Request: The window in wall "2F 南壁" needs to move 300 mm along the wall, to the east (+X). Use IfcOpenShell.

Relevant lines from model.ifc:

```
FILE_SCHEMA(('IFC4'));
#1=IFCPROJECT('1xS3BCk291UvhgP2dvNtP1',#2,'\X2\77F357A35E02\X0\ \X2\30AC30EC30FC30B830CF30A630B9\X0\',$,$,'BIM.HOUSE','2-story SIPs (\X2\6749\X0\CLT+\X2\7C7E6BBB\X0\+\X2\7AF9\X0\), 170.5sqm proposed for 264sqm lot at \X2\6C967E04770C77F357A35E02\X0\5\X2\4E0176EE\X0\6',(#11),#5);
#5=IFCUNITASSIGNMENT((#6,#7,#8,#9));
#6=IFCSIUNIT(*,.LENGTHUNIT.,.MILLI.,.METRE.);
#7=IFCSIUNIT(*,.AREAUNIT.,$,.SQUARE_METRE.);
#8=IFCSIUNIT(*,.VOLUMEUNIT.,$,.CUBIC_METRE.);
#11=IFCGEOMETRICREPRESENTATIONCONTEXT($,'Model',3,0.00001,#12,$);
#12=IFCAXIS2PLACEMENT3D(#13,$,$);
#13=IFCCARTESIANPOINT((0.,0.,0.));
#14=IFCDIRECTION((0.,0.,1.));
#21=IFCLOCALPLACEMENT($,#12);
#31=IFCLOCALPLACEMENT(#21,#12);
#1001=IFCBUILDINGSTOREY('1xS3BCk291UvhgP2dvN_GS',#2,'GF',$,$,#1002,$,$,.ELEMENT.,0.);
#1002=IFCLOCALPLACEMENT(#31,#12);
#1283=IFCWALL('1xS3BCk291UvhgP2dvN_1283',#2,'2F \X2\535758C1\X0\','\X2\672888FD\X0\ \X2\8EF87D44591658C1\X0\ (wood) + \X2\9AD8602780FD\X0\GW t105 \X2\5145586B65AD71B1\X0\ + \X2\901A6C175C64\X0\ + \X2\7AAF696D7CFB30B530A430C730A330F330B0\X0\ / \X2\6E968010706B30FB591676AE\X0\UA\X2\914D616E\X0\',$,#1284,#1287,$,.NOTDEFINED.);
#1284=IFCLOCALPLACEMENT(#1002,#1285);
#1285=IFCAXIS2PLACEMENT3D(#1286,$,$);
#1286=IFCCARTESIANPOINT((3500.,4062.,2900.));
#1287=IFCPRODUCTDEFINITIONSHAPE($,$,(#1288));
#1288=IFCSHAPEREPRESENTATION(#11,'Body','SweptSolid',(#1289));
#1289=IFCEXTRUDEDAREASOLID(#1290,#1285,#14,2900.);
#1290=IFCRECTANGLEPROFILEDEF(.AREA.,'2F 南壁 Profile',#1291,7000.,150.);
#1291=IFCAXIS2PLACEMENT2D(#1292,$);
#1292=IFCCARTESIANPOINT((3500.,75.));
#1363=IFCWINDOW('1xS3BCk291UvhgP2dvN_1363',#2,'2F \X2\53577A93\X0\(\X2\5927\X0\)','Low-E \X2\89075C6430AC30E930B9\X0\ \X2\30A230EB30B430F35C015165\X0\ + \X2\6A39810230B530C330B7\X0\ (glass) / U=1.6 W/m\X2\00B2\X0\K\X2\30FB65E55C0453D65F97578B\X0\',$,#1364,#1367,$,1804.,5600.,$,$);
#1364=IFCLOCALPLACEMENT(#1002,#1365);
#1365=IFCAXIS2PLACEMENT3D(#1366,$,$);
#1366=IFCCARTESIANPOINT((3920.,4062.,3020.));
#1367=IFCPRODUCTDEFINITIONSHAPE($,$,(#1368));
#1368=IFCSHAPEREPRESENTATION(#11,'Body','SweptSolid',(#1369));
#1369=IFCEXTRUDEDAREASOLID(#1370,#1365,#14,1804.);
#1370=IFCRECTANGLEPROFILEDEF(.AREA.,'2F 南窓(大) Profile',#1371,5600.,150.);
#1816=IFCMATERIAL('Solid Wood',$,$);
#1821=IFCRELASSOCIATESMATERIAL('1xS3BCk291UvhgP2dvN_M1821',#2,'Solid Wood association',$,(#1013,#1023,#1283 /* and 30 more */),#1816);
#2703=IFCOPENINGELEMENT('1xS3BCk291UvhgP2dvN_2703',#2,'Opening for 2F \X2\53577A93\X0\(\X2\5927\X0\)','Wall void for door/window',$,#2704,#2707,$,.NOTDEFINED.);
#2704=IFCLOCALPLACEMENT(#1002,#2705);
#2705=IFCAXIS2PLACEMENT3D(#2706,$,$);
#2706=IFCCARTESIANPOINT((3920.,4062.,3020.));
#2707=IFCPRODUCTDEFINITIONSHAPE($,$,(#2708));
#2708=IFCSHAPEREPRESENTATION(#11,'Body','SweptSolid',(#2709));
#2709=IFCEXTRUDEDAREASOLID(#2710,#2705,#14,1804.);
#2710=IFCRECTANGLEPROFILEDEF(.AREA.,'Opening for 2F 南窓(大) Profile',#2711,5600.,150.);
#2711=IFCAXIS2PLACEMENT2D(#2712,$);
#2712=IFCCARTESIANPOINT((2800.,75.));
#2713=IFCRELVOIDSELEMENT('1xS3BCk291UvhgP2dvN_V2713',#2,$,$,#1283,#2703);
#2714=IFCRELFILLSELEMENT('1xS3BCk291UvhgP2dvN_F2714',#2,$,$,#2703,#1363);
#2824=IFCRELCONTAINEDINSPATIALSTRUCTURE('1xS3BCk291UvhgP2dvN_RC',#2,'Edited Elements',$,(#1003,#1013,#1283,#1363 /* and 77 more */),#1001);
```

```python
import ifcopenshell
import ifcopenshell.api.geometry
import ifcopenshell.util.placement
import ifcopenshell.util.unit

model = ifcopenshell.open("model.ifc")
unit_scale = ifcopenshell.util.unit.calculate_unit_scale(model)

window = model.by_id(1363)
opening = window.FillsVoids[0].RelatingOpeningElement
wall = opening.VoidsElements[0].RelatingBuildingElement

wall_matrix = ifcopenshell.util.placement.get_local_placement(wall.ObjectPlacement)
shift = wall_matrix[:3, 0] * 0.3 / unit_scale
before = ifcopenshell.util.placement.get_local_placement(window.ObjectPlacement)[:3, 3].copy()

# The window is not placed relative to its opening, so move both.
for product in (opening, window):
    matrix = ifcopenshell.util.placement.get_local_placement(product.ObjectPlacement)
    matrix[:3, 3] += shift
    ifcopenshell.api.geometry.edit_object_placement(model, product=product, matrix=matrix, is_si=False)

after = ifcopenshell.util.placement.get_local_placement(window.ObjectPlacement)[:3, 3]
print("window moved by", (after - before).round(3) + 0.0)

model.write("model_edited.ifc")
```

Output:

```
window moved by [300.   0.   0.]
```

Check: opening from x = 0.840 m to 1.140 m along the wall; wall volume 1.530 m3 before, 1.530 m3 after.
